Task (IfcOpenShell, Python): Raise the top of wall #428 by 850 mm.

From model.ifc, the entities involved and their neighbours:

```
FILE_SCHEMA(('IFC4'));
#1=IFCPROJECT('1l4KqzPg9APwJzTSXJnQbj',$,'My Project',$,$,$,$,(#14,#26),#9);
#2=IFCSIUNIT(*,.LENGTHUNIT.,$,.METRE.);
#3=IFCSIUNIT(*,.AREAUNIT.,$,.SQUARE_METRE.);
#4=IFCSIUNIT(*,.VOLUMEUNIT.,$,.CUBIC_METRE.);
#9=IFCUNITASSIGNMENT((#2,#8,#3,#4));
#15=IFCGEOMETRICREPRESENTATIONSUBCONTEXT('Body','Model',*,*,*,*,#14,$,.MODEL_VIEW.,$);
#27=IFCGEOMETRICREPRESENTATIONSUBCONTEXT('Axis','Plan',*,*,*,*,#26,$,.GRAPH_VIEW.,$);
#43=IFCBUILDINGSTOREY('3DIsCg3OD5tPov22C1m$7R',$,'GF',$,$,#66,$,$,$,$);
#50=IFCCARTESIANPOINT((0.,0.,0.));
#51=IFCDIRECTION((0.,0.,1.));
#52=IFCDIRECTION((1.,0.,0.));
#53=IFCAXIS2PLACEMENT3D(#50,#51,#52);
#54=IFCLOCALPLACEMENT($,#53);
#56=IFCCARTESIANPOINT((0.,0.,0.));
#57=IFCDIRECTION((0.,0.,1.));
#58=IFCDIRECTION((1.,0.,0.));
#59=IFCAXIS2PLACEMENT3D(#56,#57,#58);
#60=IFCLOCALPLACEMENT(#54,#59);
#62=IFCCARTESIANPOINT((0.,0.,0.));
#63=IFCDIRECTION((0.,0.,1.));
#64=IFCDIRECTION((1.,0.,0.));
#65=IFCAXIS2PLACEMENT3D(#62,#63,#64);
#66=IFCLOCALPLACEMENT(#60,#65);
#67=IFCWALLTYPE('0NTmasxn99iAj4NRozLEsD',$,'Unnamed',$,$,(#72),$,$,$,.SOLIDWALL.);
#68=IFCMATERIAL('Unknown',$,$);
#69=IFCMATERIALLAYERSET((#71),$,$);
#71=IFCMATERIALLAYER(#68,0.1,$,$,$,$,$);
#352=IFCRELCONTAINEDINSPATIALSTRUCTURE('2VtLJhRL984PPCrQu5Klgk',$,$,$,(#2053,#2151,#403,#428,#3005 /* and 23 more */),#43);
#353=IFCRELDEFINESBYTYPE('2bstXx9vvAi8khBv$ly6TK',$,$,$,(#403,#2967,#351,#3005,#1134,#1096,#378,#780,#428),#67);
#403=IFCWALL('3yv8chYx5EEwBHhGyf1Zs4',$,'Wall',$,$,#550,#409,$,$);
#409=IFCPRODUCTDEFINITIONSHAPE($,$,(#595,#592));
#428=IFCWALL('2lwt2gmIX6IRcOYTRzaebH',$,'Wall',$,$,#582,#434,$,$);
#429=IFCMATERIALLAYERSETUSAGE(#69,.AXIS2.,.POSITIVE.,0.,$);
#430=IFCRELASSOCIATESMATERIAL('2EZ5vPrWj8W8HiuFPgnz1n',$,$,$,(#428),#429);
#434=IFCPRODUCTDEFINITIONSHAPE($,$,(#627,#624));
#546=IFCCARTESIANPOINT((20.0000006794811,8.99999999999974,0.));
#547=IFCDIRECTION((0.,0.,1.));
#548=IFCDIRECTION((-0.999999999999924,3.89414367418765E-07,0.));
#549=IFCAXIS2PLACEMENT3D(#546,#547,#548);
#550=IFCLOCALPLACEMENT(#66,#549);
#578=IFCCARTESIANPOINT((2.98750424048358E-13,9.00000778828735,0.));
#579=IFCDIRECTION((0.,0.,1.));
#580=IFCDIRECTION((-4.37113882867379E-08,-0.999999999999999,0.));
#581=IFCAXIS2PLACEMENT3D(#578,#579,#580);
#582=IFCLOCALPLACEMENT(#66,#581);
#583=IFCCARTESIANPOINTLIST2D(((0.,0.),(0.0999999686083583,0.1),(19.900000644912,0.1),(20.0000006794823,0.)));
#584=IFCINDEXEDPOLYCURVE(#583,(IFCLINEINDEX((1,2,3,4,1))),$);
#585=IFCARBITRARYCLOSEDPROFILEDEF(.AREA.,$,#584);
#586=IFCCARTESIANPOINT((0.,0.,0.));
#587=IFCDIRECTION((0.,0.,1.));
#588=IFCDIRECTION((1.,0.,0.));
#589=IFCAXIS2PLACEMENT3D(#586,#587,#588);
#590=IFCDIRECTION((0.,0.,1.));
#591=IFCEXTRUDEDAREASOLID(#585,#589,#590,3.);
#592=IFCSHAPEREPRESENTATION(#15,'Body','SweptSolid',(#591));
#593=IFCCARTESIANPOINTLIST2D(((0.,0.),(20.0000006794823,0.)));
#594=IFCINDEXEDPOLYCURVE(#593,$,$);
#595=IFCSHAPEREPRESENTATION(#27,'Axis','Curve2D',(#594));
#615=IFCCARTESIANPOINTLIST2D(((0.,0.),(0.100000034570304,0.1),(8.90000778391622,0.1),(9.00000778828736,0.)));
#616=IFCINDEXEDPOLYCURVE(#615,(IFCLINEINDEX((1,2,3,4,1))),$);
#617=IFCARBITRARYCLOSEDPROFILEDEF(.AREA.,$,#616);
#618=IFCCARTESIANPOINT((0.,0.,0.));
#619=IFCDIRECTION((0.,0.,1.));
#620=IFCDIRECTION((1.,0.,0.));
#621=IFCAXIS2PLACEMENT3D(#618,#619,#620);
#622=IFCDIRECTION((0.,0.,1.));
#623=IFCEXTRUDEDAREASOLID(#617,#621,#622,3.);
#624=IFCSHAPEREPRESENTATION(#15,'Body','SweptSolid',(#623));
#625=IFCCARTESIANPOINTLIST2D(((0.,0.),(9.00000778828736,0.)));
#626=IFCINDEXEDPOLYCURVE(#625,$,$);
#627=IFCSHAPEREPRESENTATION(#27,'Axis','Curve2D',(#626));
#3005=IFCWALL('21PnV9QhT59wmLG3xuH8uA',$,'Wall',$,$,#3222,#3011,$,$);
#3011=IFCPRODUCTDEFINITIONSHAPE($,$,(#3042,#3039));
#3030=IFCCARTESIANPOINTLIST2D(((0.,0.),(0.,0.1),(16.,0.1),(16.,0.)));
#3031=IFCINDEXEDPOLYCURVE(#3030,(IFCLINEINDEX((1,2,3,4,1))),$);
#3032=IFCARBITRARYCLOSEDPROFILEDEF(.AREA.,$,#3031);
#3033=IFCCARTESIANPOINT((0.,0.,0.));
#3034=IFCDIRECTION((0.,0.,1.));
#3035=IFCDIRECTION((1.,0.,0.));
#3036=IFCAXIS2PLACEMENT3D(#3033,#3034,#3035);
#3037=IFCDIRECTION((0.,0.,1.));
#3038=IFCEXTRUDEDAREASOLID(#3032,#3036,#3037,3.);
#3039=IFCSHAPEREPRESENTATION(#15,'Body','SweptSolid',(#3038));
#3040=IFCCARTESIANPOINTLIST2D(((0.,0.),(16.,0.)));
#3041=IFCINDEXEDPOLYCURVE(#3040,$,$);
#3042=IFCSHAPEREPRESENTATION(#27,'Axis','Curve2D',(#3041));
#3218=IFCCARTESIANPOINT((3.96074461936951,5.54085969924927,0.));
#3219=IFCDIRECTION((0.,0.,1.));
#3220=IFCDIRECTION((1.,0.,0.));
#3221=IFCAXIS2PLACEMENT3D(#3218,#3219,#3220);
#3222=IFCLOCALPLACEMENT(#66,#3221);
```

```python
import ifcopenshell
import ifcopenshell.geom
import ifcopenshell.util.representation
import ifcopenshell.util.shape
import ifcopenshell.util.unit

model = ifcopenshell.open("model.ifc")
unit_scale = ifcopenshell.util.unit.calculate_unit_scale(model)
settings = ifcopenshell.geom.settings()


def volume(element):
    """Net volume in cubic metres, openings subtracted."""
    shape = ifcopenshell.geom.create_shape(settings, element)
    return ifcopenshell.util.shape.get_volume(shape.geometry)


wall = model.by_guid("2lwt2gmIX6IRcOYTRzaebH")
before = volume(wall)

body = ifcopenshell.util.representation.get_representation(wall, "Model", "Body")
solid = body.Items[0]
old_height = solid.Depth
solid.Depth += 0.85 / unit_scale
after = volume(wall)

print(f"height {old_height:g} -> {solid.Depth:g}, volume {before:.3f} -> {after:.3f} m3")

model.write("model-out.ifc")
```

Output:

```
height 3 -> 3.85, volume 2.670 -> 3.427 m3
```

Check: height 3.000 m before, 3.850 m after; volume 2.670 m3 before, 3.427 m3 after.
